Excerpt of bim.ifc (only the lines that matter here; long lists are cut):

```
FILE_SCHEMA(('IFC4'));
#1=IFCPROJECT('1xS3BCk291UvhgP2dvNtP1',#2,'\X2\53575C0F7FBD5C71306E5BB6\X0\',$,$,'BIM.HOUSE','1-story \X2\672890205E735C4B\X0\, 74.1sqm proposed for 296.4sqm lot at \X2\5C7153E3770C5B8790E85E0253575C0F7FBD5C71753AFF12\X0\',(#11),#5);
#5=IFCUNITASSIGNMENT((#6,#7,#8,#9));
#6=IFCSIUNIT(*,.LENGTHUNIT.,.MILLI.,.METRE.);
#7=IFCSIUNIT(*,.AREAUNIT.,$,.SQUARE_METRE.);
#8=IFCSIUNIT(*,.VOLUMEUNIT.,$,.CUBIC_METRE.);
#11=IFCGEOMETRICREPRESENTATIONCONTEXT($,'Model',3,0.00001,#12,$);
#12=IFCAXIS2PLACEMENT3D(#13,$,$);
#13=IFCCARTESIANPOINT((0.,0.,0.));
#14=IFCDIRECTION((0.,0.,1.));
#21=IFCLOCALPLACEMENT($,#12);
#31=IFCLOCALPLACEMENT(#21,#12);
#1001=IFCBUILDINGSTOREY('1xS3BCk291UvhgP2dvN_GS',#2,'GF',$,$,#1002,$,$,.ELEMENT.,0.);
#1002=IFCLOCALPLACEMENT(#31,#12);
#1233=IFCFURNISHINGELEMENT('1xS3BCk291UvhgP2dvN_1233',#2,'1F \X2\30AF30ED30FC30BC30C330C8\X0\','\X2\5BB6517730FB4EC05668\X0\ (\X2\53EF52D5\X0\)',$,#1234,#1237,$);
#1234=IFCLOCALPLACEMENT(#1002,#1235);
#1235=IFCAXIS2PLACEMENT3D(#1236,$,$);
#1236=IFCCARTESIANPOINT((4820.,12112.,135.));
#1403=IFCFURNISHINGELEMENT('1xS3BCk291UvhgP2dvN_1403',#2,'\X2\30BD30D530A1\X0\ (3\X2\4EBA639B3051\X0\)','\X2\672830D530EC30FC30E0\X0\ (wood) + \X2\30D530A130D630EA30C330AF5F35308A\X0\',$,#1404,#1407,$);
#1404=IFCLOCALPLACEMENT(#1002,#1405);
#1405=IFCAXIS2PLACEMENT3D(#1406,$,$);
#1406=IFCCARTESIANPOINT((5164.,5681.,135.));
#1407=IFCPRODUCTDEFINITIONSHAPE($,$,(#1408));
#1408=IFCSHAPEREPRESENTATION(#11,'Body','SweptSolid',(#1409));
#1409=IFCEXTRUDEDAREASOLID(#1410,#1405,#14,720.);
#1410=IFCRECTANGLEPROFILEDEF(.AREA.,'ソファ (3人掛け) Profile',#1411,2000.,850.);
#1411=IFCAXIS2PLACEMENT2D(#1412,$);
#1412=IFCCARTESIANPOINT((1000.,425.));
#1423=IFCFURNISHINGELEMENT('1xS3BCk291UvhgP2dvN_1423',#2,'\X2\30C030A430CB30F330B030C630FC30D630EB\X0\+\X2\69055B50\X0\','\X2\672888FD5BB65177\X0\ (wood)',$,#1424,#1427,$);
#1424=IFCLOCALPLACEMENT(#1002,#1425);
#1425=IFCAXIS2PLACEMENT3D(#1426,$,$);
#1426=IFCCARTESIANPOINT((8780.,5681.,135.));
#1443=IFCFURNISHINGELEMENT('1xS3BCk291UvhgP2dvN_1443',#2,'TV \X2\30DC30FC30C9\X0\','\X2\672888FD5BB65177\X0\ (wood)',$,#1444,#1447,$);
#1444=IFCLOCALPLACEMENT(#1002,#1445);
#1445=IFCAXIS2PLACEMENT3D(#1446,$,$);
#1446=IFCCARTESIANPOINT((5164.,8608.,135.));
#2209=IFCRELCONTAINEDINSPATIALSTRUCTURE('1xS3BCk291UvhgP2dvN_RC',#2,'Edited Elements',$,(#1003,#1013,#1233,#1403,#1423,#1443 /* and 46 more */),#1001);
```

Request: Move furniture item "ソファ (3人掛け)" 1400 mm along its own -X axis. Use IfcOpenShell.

```python
import ifcopenshell
import ifcopenshell.api.geometry
import ifcopenshell.util.placement

model = ifcopenshell.open("bim.ifc")

item = model.by_guid("1xS3BCk291UvhgP2dvN_1403")
matrix = ifcopenshell.util.placement.get_local_placement(item.ObjectPlacement)
matrix[:3, 3] -= matrix[:3, 0] * 1400.0
ifcopenshell.api.geometry.edit_object_placement(model, product=item, matrix=matrix, is_si=False)

print(ifcopenshell.util.placement.get_local_placement(item.ObjectPlacement).round(3) + 0.0)

model.write("bim_rev.ifc")
```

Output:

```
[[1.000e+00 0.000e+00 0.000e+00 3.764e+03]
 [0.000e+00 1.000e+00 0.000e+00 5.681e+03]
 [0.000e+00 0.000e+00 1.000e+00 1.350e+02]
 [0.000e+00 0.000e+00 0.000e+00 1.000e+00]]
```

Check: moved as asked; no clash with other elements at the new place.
